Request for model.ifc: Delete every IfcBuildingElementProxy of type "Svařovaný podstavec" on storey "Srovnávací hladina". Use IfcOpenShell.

First a look at what the model holds.

```python
import ifcopenshell
import ifcopenshell.util.element

model = ifcopenshell.open("model.ifc")
print(model.schema)
storey = next(s for s in model.by_type("IfcBuildingStorey") if s.Name == "Srovnávací hladina")
proxies = [e for e in ifcopenshell.util.element.get_decomposition(storey) if e.is_a("IfcBuildingElementProxy")]
seen = {}
for e in proxies:
    element_type = ifcopenshell.util.element.get_type(e)
    name = element_type.Name if element_type not in (None, e) else None
    seen[name] = seen.get(name, 0) + 1
for name, count in sorted(seen.items(), key=str):
    print(count, "x", name)
```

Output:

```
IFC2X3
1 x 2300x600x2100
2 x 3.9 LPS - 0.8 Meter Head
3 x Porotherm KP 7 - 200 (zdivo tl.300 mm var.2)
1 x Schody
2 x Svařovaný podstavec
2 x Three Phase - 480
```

```python
import ifcopenshell
import ifcopenshell.api.root
import ifcopenshell.util.element

model = ifcopenshell.open("model.ifc")

storey = next(s for s in model.by_type("IfcBuildingStorey") if s.Name == "Srovnávací hladina")
proxies = [e for e in ifcopenshell.util.element.get_decomposition(storey) if e.is_a("IfcBuildingElementProxy")]
targets = [e for e in proxies if (t := ifcopenshell.util.element.get_type(e)) not in (None, e) and t.Name == "Svařovaný podstavec"]

for e in targets:
    ifcopenshell.api.root.remove_product(model, product=e)
print(len(targets), "removed")

model.write("model_v2.ifc")
```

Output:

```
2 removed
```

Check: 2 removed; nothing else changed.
